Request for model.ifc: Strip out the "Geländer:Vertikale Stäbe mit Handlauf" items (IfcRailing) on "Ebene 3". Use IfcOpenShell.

First a look at what the model holds.

```python
import ifcopenshell
import ifcopenshell.util.element

model = ifcopenshell.open("model.ifc")
print(model.schema)
storey = next(s for s in model.by_type("IfcBuildingStorey") if s.Name == "Ebene 3")
railings = [e for e in ifcopenshell.util.element.get_decomposition(storey) if e.is_a("IfcRailing")]
seen = {}
for e in railings:
    element_type = ifcopenshell.util.element.get_type(e)
    name = element_type.Name if element_type not in (None, e) else None
    seen[name] = seen.get(name, 0) + 1
for name, count in sorted(seen.items(), key=str):
    print(count, "x", name)
```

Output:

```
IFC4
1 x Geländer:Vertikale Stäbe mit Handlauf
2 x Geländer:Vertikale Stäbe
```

```python
import ifcopenshell
import ifcopenshell.api.root
import ifcopenshell.util.element

model = ifcopenshell.open("model.ifc")

storey = next(s for s in model.by_type("IfcBuildingStorey") if s.Name == "Ebene 3")
railings = [e for e in ifcopenshell.util.element.get_decomposition(storey) if e.is_a("IfcRailing")]
targets = [e for e in railings if (t := ifcopenshell.util.element.get_type(e)) not in (None, e) and t.Name == "Geländer:Vertikale Stäbe mit Handlauf"]

for e in targets:
    ifcopenshell.api.root.remove_product(model, product=e)
print(len(targets), "removed")

model.write("model_v2.ifc")
```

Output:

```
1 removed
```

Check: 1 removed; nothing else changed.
